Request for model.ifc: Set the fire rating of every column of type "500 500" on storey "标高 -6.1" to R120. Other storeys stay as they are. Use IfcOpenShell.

First a look at what the model holds.

```python
import ifcopenshell
import ifcopenshell.util.element

model = ifcopenshell.open("model.ifc")
print(model.schema)
storey = next(s for s in model.by_type("IfcBuildingStorey") if s.Name == "标高 -6.1")
columns = [e for e in ifcopenshell.util.element.get_decomposition(storey) if e.is_a("IfcColumn")]
seen = {}
for e in columns:
    element_type = ifcopenshell.util.element.get_type(e)
    key = (element_type.Name if element_type != e and element_type else None, ifcopenshell.util.element.get_pset(e, "Pset_ColumnCommon", "FireRating"))
    seen[key] = seen.get(key, 0) + 1
for (name, value), count in sorted(seen.items(), key=str):
    print(count, "x", name, "|", value)
```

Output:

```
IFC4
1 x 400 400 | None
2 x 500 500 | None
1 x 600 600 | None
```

```python
import ifcopenshell
import ifcopenshell.api.pset
import ifcopenshell.util.element

model = ifcopenshell.open("model.ifc")

storey = next(s for s in model.by_type("IfcBuildingStorey") if s.Name == "标高 -6.1")
columns = [e for e in ifcopenshell.util.element.get_decomposition(storey) if e.is_a("IfcColumn")]

count = 0
for e in columns:
    element_type = ifcopenshell.util.element.get_type(e)
    if element_type in (None, e) or element_type.Name != "500 500":
        continue
    # add_pset returns the element's existing set when there is one.
    pset = ifcopenshell.api.pset.add_pset(model, product=e, name="Pset_ColumnCommon")
    ifcopenshell.api.pset.edit_pset(model, pset=pset, properties={"FireRating": "R120"})
    count += 1

print(count, "columns updated")

model.write("model_rev.ifc")
```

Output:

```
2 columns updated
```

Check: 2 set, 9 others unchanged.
